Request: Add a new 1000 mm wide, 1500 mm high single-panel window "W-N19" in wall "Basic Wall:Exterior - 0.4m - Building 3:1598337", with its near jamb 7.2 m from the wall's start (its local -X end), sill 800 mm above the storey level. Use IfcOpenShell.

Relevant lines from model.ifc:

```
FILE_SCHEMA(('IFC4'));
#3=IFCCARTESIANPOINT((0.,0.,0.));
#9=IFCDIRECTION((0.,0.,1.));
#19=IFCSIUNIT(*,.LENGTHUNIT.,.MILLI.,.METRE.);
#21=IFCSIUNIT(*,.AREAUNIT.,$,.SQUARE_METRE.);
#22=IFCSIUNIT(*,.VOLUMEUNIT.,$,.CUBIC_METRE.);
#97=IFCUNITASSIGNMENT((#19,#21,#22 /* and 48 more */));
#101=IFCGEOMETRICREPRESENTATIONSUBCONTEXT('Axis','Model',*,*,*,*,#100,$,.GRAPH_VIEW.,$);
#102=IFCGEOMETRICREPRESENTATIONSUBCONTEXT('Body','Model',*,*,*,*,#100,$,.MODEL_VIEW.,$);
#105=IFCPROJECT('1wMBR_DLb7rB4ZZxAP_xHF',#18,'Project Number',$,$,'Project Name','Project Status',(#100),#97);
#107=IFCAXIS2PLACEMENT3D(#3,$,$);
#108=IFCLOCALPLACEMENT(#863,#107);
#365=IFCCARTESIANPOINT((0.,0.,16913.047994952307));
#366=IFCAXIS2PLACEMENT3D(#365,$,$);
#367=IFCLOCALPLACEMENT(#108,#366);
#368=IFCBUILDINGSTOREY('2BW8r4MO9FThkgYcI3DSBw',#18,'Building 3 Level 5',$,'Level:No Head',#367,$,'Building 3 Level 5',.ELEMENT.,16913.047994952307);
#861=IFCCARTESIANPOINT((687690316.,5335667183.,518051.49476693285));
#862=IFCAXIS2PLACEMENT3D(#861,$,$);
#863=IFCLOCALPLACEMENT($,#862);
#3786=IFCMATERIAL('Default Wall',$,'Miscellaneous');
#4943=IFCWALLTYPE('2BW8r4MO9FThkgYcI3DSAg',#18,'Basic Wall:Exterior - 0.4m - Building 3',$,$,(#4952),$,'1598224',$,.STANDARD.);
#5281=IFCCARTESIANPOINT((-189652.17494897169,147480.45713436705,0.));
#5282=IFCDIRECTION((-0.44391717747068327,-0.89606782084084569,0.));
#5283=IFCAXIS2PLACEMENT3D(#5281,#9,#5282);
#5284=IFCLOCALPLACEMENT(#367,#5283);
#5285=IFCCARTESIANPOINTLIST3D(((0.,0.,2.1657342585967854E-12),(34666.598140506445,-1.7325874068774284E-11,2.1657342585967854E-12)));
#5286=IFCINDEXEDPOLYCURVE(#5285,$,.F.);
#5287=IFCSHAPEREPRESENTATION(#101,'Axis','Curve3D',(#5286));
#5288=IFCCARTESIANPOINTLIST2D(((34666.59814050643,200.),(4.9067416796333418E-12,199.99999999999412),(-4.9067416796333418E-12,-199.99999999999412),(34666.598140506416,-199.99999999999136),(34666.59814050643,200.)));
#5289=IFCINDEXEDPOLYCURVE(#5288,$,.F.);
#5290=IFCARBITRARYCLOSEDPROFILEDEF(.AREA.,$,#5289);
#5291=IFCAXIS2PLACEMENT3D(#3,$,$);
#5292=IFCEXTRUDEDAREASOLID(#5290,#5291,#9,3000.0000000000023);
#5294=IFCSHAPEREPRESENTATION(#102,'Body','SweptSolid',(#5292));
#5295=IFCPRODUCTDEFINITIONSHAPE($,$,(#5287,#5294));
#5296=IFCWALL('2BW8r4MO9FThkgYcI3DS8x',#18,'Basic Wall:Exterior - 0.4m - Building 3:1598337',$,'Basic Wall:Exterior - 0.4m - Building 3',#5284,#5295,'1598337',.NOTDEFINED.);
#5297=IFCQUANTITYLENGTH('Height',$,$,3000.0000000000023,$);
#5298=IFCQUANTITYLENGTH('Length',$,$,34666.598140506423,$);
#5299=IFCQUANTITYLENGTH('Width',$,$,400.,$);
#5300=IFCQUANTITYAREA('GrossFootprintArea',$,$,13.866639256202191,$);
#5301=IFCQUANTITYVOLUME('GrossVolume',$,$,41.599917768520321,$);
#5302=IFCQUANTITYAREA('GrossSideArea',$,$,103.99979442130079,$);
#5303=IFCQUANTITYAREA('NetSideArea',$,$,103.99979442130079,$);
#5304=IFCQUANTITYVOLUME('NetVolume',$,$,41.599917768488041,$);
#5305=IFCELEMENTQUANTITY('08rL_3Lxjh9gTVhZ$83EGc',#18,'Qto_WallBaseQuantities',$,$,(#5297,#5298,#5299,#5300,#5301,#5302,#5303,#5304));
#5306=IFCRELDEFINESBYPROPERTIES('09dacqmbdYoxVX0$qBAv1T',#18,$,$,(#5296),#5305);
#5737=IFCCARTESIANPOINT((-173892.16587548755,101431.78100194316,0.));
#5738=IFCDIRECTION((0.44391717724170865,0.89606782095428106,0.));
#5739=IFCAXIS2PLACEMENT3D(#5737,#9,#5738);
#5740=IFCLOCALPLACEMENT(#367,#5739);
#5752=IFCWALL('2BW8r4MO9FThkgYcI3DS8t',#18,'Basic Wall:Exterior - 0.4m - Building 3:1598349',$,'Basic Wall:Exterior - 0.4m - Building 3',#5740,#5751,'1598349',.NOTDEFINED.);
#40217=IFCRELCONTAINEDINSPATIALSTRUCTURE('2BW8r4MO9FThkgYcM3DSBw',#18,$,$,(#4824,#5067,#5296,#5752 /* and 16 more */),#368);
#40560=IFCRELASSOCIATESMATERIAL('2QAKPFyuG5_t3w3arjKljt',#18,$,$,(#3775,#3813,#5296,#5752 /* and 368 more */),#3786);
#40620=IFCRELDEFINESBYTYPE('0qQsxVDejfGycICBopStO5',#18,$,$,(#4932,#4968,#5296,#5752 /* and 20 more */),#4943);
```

```python
import numpy as np
import ifcopenshell
import ifcopenshell.api.feature
import ifcopenshell.api.geometry
import ifcopenshell.api.pset
import ifcopenshell.api.root
import ifcopenshell.api.spatial
import ifcopenshell.geom
import ifcopenshell.util.element
import ifcopenshell.util.placement
import ifcopenshell.util.representation
import ifcopenshell.util.shape
import ifcopenshell.util.unit

model = ifcopenshell.open("model.ifc")
unit_scale = ifcopenshell.util.unit.calculate_unit_scale(model)
area_scale = ifcopenshell.util.unit.calculate_unit_scale(model, "AREAUNIT")
volume_scale = ifcopenshell.util.unit.calculate_unit_scale(model, "VOLUMEUNIT")
settings = ifcopenshell.geom.settings()


def volume(element):
    """Net volume in cubic metres, openings subtracted."""
    shape = ifcopenshell.geom.create_shape(settings, element)
    return ifcopenshell.util.shape.get_volume(shape.geometry)


wall = model.by_id(5296)
storey = ifcopenshell.util.element.get_container(wall, ifc_class="IfcBuildingStorey")
context = ifcopenshell.util.representation.get_context(model, "Model", "Body", "MODEL_VIEW")
before = volume(wall)

width, height, from_end, sill = 1, 1.5, 7.2, 0.8  # metres

# The wall runs along its own X axis, and the end named is its -X end.
wall_shape = ifcopenshell.geom.create_shape(settings, wall)
x, y, z = ifcopenshell.util.shape.get_vertices(wall_shape.geometry).T
start = x.min() + from_end
face, thickness = float(y.min()), float(y.max() - y.min())
wall_matrix = ifcopenshell.util.placement.get_local_placement(wall.ObjectPlacement)
level = ifcopenshell.util.placement.get_local_placement(storey.ObjectPlacement)[2, 3]


def in_wall(x, y):
    """Placement at x, y metres in the wall's axes, at sill height."""
    matrix = wall_matrix.copy()
    matrix[:, 3] = wall_matrix @ np.array([x / unit_scale, y / unit_scale, 0.0, 1.0])
    matrix[2, 3] = level + sill / unit_scale
    return matrix


# Opening: a box that overshoots both wall faces by 50 mm.
opening = ifcopenshell.api.root.create_entity(model, ifc_class="IfcOpeningElement", predefined_type="OPENING")
box = ifcopenshell.api.geometry.add_wall_representation(
    model, context=context, length=width, height=height, thickness=thickness + 0.1
)
ifcopenshell.api.geometry.assign_representation(model, product=opening, representation=box)
ifcopenshell.api.geometry.edit_object_placement(model, product=opening, matrix=in_wall(start, face - 0.05), is_si=False)
ifcopenshell.api.feature.add_feature(model, feature=opening, element=wall)

window = ifcopenshell.api.root.create_entity(model, ifc_class="IfcWindow", name="W-N19", predefined_type="WINDOW")
window.OverallWidth, window.OverallHeight = width / unit_scale, height / unit_scale
window.PartitioningType = "SINGLE_PANEL"
body = ifcopenshell.api.geometry.add_window_representation(
    model,
    context=context,
    overall_width=window.OverallWidth,
    overall_height=window.OverallHeight,
    partition_type="SINGLE_PANEL",
)
ifcopenshell.api.geometry.assign_representation(model, product=window, representation=body)
ifcopenshell.api.spatial.assign_container(model, products=[window], relating_structure=storey)
ifcopenshell.api.feature.add_filling(model, opening=opening, element=window)

# Centre the window in the wall's thickness.
ifcopenshell.api.geometry.edit_object_placement(model, product=window, matrix=in_wall(start, face), is_si=False)
window_shape = ifcopenshell.geom.create_shape(settings, window)
depth = ifcopenshell.util.shape.get_vertices(window_shape.geometry)[:, 1]
offset = face + thickness / 2 - (depth.min() + depth.max()) / 2
ifcopenshell.api.geometry.edit_object_placement(model, product=window, matrix=in_wall(start, offset), is_si=False)

after = volume(wall)

# Update the wall's stored quantities.
qto = model.by_id(ifcopenshell.util.element.get_pset(wall, "Qto_WallBaseQuantities", should_inherit=False)["id"])
ifcopenshell.api.pset.edit_qto(model, qto=qto, properties={
    "NetSideArea": after / thickness / area_scale,
    "NetVolume": after / volume_scale,
})

print(f"wall volume {before:.3f} -> {after:.3f} m3")

model.write("model-out.ifc")
```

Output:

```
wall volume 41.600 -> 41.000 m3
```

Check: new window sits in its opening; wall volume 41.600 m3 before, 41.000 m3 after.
